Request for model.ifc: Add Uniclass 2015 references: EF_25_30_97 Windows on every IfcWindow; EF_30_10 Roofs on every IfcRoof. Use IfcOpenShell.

First a look at what the model holds.

```python
import ifcopenshell

model = ifcopenshell.open("model.ifc")
print(model.schema)
print("classifications:", [c.Name for c in model.by_type("IfcClassification")])
for ifc_class in ("IfcDoor", "IfcRoof", "IfcStair", "IfcWall", "IfcWindow"):
    print(ifc_class, len(model.by_type(ifc_class)))
```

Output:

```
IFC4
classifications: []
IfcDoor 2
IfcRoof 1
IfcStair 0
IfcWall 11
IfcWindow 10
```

```python
import ifcopenshell
import ifcopenshell.api.classification

model = ifcopenshell.open("model.ifc")

system = ifcopenshell.api.classification.add_classification(model, classification="Uniclass 2015")

codes = {
    "IfcWindow": ("EF_25_30_97", "Windows"),
    "IfcRoof": ("EF_30_10", "Roofs"),
}
for ifc_class, (code, name) in codes.items():
    products = model.by_type(ifc_class)
    ifcopenshell.api.classification.add_reference(
        model, products=products, classification=system, identification=code, name=name
    )
    print(code, len(products))

model.write("model_rev.ifc")
```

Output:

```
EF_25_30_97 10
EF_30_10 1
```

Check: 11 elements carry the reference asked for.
